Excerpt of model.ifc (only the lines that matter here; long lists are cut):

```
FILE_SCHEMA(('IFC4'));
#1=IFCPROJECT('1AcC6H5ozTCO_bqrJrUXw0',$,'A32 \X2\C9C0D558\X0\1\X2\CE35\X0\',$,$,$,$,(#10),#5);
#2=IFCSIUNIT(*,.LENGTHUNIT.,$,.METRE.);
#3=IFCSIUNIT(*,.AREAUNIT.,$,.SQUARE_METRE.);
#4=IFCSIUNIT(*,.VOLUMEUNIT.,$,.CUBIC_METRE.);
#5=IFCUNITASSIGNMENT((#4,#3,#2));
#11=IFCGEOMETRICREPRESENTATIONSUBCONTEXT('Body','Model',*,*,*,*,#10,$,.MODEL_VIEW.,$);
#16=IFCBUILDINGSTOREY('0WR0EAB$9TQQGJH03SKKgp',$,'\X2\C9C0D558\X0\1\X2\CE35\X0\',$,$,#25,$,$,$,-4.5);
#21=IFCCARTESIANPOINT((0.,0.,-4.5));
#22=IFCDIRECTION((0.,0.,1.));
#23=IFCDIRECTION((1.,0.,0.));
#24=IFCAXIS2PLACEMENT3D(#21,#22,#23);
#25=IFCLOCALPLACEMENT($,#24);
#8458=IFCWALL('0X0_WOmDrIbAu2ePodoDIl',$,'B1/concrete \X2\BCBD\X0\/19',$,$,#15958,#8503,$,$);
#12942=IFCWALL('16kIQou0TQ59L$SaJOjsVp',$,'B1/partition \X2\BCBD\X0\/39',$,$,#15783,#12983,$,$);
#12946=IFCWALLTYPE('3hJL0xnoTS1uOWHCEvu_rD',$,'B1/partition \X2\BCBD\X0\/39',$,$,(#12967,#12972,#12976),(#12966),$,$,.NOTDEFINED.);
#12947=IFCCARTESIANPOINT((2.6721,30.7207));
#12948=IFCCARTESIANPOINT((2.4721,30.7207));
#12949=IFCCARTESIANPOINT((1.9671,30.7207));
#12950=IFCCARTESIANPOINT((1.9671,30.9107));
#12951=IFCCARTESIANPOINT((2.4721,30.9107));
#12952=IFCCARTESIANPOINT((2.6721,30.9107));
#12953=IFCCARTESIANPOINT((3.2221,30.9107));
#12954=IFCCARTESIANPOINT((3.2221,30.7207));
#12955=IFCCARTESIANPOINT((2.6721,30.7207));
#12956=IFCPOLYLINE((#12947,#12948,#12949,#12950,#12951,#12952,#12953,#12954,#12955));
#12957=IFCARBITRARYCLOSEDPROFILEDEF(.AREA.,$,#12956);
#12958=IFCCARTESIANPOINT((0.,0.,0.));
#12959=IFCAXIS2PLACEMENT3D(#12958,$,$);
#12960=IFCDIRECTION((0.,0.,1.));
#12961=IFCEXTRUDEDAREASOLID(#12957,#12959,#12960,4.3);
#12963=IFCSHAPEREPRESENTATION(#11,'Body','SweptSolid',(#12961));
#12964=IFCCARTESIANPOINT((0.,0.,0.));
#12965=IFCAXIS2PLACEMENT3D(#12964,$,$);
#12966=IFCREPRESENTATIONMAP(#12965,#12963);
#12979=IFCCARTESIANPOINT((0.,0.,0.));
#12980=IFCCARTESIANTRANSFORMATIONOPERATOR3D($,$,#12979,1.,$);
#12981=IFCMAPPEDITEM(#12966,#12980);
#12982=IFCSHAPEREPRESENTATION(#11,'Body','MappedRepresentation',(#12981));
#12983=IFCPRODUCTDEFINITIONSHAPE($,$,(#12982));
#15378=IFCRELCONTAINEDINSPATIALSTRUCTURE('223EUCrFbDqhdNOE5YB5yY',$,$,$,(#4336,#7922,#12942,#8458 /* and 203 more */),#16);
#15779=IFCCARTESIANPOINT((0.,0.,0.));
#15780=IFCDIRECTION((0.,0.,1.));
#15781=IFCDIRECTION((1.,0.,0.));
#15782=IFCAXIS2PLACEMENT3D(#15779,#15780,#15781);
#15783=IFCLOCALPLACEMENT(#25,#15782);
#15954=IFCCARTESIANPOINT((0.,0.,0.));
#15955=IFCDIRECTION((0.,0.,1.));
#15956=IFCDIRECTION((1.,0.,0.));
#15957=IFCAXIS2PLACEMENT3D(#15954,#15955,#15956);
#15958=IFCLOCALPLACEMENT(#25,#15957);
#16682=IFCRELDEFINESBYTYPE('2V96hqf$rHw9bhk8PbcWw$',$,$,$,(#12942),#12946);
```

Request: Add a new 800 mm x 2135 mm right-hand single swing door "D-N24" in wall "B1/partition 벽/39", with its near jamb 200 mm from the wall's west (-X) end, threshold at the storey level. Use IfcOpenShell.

```python
import numpy as np
import ifcopenshell
import ifcopenshell.api.feature
import ifcopenshell.api.geometry
import ifcopenshell.api.root
import ifcopenshell.api.spatial
import ifcopenshell.geom
import ifcopenshell.util.element
import ifcopenshell.util.placement
import ifcopenshell.util.representation
import ifcopenshell.util.shape
import ifcopenshell.util.unit

model = ifcopenshell.open("model.ifc")
unit_scale = ifcopenshell.util.unit.calculate_unit_scale(model)
settings = ifcopenshell.geom.settings()


def volume(element):
    """Net volume in cubic metres, openings subtracted."""
    shape = ifcopenshell.geom.create_shape(settings, element)
    return ifcopenshell.util.shape.get_volume(shape.geometry)


wall = model.by_guid("16kIQou0TQ59L$SaJOjsVp")
storey = ifcopenshell.util.element.get_container(wall, ifc_class="IfcBuildingStorey")
context = ifcopenshell.util.representation.get_context(model, "Model", "Body", "MODEL_VIEW")
before = volume(wall)

width, height, from_end, sill = 0.8, 2.135, 0.2, 0.0  # metres

# The wall runs along its own X axis, and the end named is its -X end.
wall_shape = ifcopenshell.geom.create_shape(settings, wall)
x, y, z = ifcopenshell.util.shape.get_vertices(wall_shape.geometry).T
start = x.min() + from_end
face, thickness = float(y.min()), float(y.max() - y.min())
wall_matrix = ifcopenshell.util.placement.get_local_placement(wall.ObjectPlacement)
level = ifcopenshell.util.placement.get_local_placement(storey.ObjectPlacement)[2, 3]


def in_wall(x, y):
    """Placement at x, y metres in the wall's axes, at sill height."""
    matrix = wall_matrix.copy()
    matrix[:, 3] = wall_matrix @ np.array([x / unit_scale, y / unit_scale, 0.0, 1.0])
    matrix[2, 3] = level + sill / unit_scale
    return matrix


# Opening: a box that overshoots both wall faces by 50 mm.
opening = ifcopenshell.api.root.create_entity(model, ifc_class="IfcOpeningElement", predefined_type="OPENING")
box = ifcopenshell.api.geometry.add_wall_representation(
    model, context=context, length=width, height=height, thickness=thickness + 0.1
)
ifcopenshell.api.geometry.assign_representation(model, product=opening, representation=box)
ifcopenshell.api.geometry.edit_object_placement(model, product=opening, matrix=in_wall(start, face - 0.05), is_si=False)
ifcopenshell.api.feature.add_feature(model, feature=opening, element=wall)

door = ifcopenshell.api.root.create_entity(model, ifc_class="IfcDoor", name="D-N24", predefined_type="DOOR")
door.OverallWidth, door.OverallHeight = width / unit_scale, height / unit_scale
door.OperationType = "SINGLE_SWING_RIGHT"
body = ifcopenshell.api.geometry.add_door_representation(
    model,
    context=context,
    overall_width=door.OverallWidth,
    overall_height=door.OverallHeight,
    operation_type="SINGLE_SWING_RIGHT",
    lining_properties={"LiningDepth": thickness / unit_scale, "ThresholdDepth": thickness / unit_scale},
)
ifcopenshell.api.geometry.assign_representation(model, product=door, representation=body)
ifcopenshell.api.spatial.assign_container(model, products=[door], relating_structure=storey)
ifcopenshell.api.feature.add_filling(model, opening=opening, element=door)

# The lining spans the wall, so the door starts at the wall face.
ifcopenshell.api.geometry.edit_object_placement(model, product=door, matrix=in_wall(start, face), is_si=False)

after = volume(wall)

print(f"wall volume {before:.3f} -> {after:.3f} m3")

model.write("model_v2.ifc")
```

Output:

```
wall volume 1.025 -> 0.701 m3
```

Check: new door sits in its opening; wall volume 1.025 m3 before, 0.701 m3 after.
